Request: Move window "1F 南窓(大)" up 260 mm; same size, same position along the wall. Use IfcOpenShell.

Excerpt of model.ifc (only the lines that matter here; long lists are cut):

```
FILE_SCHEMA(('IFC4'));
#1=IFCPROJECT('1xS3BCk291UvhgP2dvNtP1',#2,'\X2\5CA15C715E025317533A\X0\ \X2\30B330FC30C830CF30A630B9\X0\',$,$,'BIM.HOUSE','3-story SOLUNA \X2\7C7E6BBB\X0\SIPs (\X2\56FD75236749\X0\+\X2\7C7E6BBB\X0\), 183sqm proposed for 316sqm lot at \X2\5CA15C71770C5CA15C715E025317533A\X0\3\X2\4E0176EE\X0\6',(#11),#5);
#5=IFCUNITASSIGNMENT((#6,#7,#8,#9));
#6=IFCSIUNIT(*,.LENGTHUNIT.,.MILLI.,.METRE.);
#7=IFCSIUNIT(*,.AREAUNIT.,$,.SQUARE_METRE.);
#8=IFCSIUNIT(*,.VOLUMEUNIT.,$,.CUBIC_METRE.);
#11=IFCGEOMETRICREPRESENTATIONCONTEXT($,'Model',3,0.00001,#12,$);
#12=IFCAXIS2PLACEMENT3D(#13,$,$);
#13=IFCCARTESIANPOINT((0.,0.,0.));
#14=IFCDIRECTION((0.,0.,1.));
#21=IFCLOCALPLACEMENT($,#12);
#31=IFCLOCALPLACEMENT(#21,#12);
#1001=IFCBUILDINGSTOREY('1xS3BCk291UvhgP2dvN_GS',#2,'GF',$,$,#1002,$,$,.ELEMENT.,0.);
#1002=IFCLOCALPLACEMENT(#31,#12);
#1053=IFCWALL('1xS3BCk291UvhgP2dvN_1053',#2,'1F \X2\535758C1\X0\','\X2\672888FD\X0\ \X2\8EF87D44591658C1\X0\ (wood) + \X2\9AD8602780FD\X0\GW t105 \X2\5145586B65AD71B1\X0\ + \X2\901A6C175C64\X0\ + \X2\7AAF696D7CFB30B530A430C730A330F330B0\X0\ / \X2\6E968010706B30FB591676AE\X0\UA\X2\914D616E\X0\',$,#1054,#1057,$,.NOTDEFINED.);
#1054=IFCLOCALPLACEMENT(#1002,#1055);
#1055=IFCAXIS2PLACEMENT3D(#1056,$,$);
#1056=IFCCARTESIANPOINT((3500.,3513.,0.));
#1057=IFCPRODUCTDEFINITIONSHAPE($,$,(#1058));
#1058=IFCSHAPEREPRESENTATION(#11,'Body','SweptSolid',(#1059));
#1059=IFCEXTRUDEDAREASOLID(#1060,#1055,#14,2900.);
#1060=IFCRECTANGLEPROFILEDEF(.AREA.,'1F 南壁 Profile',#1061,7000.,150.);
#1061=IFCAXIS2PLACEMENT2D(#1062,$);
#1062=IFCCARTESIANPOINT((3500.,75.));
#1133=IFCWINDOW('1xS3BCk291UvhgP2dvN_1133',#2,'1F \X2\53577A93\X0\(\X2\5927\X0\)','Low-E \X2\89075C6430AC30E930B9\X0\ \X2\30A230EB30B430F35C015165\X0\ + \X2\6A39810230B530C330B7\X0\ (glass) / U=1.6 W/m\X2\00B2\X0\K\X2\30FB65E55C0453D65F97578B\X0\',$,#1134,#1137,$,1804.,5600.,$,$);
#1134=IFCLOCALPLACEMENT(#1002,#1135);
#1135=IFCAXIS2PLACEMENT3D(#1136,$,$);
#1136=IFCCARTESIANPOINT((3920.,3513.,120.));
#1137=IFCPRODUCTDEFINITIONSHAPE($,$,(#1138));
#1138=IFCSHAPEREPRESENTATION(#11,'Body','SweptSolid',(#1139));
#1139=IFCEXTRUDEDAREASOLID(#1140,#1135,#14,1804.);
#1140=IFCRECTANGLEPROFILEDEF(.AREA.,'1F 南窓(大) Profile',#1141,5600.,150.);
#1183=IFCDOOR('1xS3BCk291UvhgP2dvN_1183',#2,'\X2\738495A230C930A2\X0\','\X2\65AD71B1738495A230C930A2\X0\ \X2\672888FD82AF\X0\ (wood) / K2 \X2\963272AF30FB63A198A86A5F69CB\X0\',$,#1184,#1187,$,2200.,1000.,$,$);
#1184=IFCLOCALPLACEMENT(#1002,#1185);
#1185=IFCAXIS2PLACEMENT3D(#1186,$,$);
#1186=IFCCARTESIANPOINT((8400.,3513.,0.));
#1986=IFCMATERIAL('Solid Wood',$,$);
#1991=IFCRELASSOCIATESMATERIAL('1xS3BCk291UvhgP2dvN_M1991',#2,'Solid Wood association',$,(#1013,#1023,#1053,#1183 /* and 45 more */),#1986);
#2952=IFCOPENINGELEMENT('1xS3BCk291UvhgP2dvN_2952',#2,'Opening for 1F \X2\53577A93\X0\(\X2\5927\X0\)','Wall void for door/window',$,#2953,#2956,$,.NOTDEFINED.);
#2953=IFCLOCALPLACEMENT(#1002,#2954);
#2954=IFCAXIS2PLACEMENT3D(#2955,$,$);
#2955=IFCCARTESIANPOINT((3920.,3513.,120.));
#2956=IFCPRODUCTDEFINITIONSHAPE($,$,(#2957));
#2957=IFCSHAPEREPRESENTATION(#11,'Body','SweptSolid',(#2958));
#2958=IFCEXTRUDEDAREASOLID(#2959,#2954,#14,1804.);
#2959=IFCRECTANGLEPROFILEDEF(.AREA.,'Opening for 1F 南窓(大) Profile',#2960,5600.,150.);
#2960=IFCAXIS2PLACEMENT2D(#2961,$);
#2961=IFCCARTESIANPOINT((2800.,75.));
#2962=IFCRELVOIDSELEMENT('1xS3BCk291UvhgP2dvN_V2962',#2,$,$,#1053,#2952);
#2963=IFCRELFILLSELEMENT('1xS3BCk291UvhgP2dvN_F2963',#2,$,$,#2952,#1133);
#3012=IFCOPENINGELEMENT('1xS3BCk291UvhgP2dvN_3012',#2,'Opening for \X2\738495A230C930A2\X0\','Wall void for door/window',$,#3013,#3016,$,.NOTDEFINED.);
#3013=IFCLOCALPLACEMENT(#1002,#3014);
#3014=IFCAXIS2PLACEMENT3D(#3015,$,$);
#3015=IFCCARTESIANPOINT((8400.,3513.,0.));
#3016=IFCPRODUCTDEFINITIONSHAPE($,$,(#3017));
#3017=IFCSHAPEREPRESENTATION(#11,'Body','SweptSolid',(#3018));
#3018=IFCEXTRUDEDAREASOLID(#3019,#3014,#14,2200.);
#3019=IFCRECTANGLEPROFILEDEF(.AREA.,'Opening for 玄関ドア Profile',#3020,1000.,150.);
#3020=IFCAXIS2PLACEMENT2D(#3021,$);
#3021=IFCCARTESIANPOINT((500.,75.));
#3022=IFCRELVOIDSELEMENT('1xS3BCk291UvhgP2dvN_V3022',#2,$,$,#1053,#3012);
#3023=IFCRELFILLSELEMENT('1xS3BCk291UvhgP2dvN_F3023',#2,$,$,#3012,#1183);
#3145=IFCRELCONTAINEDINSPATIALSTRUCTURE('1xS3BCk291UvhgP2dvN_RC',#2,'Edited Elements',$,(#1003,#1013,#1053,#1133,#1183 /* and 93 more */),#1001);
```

```python
import numpy as np
import ifcopenshell
import ifcopenshell.api.geometry
import ifcopenshell.util.placement
import ifcopenshell.util.unit

model = ifcopenshell.open("model.ifc")
unit_scale = ifcopenshell.util.unit.calculate_unit_scale(model)

window = model.by_id(1133)
opening = window.FillsVoids[0].RelatingOpeningElement
dz = 260.0

shift = np.array([0.0, 0.0, dz])
# The window is not placed relative to its opening, so move both.
for product in (opening, window):
    matrix = ifcopenshell.util.placement.get_local_placement(product.ObjectPlacement)
    matrix[:3, 3] += shift
    ifcopenshell.api.geometry.edit_object_placement(model, product=product, matrix=matrix, is_si=False)

print(f"moved by {dz * unit_scale:+.3f} m")

model.write("model-out.ifc")
```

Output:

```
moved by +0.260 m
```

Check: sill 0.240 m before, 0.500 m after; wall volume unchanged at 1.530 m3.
